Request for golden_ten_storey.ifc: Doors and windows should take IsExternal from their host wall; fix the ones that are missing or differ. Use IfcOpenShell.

First a look at what the model holds.

```python
import ifcopenshell
import ifcopenshell.util.element

model = ifcopenshell.open("golden_ten_storey.ifc")
print(model.schema)
seen = {}
for e in model.by_type("IfcDoor") + model.by_type("IfcWindow"):
    if not e.FillsVoids:
        continue
    host = e.FillsVoids[0].RelatingOpeningElement.VoidsElements[0].RelatingBuildingElement
    own = ifcopenshell.util.element.get_pset(e, f"Pset_{e.is_a()[3:].removesuffix('StandardCase')}Common", "IsExternal")
    wall = ifcopenshell.util.element.get_pset(host, "Pset_WallCommon", "IsExternal")
    seen[e.is_a(), own, wall] = seen.get((e.is_a(), own, wall), 0) + 1
for (cls, own, wall), count in sorted(seen.items(), key=str):
    print(count, cls, "IsExternal:", own, "| host wall:", wall)
```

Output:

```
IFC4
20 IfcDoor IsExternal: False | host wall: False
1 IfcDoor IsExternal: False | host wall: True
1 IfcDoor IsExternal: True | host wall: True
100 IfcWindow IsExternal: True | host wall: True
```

```python
import ifcopenshell
import ifcopenshell.api.pset
import ifcopenshell.util.element

model = ifcopenshell.open("golden_ten_storey.ifc")

count = 0
for ifc_class, pset_name in (("IfcDoor", "Pset_DoorCommon"), ("IfcWindow", "Pset_WindowCommon")):
    for e in model.by_type(ifc_class):
        if not e.FillsVoids:
            continue
        host = e.FillsVoids[0].RelatingOpeningElement.VoidsElements[0].RelatingBuildingElement
        external = ifcopenshell.util.element.get_pset(host, "Pset_WallCommon", "IsExternal")
        if external is None or ifcopenshell.util.element.get_pset(e, pset_name, "IsExternal") == external:
            continue
        pset = ifcopenshell.api.pset.add_pset(model, product=e, name=pset_name)
        ifcopenshell.api.pset.edit_pset(model, pset=pset, properties={"IsExternal": external})
        count += 1

print(count, "updated")

model.write("golden_ten_storey_edited.ifc")
```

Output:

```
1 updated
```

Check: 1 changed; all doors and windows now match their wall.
